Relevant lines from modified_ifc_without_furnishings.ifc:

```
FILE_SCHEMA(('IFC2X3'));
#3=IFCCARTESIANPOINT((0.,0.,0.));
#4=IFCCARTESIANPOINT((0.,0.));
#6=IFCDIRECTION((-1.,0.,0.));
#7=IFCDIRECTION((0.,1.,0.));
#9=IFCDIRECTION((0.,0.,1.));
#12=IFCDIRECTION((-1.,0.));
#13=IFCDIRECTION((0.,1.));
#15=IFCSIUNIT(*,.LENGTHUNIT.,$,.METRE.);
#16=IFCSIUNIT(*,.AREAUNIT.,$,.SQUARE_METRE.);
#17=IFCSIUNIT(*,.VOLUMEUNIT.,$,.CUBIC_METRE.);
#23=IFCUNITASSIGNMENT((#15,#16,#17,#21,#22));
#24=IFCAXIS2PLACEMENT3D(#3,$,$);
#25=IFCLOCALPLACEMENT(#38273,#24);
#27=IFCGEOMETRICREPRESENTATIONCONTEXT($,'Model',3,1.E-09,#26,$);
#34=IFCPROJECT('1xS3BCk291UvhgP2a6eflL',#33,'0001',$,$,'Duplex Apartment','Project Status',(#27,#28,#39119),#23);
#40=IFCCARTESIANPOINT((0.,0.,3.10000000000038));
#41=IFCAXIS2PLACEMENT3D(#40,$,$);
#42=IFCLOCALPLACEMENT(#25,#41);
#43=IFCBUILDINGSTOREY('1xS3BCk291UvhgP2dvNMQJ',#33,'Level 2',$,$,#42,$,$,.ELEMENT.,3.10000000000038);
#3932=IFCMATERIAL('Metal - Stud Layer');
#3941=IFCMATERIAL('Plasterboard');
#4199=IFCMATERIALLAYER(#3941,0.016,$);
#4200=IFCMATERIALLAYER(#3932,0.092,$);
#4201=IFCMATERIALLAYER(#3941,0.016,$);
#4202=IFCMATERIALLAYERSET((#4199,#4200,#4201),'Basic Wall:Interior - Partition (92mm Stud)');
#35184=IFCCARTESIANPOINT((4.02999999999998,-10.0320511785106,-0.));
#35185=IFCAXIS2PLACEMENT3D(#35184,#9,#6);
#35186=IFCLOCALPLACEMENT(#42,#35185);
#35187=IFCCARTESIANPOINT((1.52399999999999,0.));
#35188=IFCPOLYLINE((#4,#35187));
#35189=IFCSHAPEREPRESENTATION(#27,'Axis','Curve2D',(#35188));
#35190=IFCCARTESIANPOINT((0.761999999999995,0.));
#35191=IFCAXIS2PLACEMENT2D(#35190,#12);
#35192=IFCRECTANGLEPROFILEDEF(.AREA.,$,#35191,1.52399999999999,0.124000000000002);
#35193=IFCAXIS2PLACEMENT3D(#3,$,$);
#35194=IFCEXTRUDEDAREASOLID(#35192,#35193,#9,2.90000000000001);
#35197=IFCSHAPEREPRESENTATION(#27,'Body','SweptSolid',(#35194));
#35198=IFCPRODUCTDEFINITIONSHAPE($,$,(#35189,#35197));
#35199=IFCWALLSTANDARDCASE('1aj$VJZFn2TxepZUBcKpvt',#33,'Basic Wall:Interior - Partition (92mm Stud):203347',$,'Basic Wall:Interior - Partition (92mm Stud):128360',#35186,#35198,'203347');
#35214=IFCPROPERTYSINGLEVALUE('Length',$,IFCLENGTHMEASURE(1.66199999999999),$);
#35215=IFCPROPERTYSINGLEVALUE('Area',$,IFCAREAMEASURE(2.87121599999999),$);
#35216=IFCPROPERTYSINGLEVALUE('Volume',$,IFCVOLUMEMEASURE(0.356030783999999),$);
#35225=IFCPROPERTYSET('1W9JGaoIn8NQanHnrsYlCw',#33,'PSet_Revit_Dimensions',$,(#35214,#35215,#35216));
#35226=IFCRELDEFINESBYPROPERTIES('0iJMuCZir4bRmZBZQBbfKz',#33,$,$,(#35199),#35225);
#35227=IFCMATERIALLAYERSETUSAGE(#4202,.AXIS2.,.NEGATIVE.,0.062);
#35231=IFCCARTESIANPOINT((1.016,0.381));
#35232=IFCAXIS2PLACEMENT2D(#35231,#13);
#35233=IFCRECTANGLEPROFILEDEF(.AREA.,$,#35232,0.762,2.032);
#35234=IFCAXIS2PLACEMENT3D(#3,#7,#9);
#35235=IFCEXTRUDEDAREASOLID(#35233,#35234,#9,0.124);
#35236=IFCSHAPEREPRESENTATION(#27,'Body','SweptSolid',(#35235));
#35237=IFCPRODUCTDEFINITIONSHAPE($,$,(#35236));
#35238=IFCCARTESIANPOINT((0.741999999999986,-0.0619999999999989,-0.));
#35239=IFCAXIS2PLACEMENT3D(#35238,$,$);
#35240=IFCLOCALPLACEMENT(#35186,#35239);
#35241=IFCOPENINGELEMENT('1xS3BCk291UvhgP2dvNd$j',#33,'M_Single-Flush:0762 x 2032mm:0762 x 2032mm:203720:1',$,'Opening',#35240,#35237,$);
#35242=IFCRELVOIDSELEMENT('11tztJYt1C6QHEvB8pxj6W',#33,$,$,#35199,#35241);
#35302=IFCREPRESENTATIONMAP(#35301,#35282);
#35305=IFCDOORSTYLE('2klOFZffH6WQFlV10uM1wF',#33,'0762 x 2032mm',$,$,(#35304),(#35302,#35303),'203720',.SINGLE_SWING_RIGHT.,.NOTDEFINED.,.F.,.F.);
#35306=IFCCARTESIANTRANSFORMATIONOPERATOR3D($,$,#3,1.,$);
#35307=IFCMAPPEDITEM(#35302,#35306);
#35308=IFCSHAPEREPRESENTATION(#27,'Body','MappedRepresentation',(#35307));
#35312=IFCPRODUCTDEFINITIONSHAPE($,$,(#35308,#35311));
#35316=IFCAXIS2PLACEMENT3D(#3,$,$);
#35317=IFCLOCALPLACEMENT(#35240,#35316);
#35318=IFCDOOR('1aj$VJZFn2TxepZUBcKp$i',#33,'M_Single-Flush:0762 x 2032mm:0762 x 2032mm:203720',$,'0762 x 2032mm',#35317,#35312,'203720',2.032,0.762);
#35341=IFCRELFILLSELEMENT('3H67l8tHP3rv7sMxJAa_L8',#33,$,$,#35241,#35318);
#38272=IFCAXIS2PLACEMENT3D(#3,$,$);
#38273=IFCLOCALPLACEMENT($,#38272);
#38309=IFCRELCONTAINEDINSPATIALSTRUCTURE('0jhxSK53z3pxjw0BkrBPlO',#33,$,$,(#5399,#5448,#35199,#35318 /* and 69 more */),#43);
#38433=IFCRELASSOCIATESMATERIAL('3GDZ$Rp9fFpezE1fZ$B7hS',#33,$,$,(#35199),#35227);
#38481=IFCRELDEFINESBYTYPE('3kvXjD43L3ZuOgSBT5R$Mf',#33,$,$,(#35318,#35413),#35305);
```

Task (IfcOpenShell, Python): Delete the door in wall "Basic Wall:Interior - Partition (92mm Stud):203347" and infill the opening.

```python
import ifcopenshell
import ifcopenshell.api.feature
import ifcopenshell.api.pset
import ifcopenshell.api.root
import ifcopenshell.geom
import ifcopenshell.util.element
import ifcopenshell.util.shape
import ifcopenshell.util.unit

model = ifcopenshell.open("modified_ifc_without_furnishings.ifc")
area_scale = ifcopenshell.util.unit.calculate_unit_scale(model, "AREAUNIT")
volume_scale = ifcopenshell.util.unit.calculate_unit_scale(model, "VOLUMEUNIT")
settings = ifcopenshell.geom.settings()


def volume(element):
    """Net volume in cubic metres, openings subtracted."""
    shape = ifcopenshell.geom.create_shape(settings, element)
    return ifcopenshell.util.shape.get_volume(shape.geometry)


door = model.by_guid("1aj$VJZFn2TxepZUBcKp$i")
opening = door.FillsVoids[0].RelatingOpeningElement
wall = opening.VoidsElements[0].RelatingBuildingElement
before = volume(wall)

ifcopenshell.api.root.remove_product(model, product=door)
ifcopenshell.api.feature.remove_feature(model, feature=opening)

after = volume(wall)
thickness = 0.124  # wall thickness in metres

# Update the wall's stored quantities.
pset = model.by_id(ifcopenshell.util.element.get_pset(wall, "PSet_Revit_Dimensions", should_inherit=False)["id"])
ifcopenshell.api.pset.edit_pset(model, pset=pset, properties={
    "Area": model.create_entity("IfcAreaMeasure", after / thickness / area_scale),
    "Volume": model.create_entity("IfcVolumeMeasure", after / volume_scale),
})

print(f"wall volume {before:.3f} -> {after:.3f} m3")

model.write("modified_ifc_without_furnishings-out.ifc")
```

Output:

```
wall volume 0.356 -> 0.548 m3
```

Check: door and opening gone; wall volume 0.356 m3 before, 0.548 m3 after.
